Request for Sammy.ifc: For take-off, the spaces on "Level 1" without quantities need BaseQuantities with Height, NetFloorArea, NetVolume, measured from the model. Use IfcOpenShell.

First a look at what the model holds.

```python
import ifcopenshell
import ifcopenshell.util.element
import ifcopenshell.util.unit

model = ifcopenshell.open("Sammy.ifc")
print(model.schema)
for unit_type in ("LENGTHUNIT", "AREAUNIT", "VOLUMEUNIT"):
    print(unit_type, ifcopenshell.util.unit.calculate_unit_scale(model, unit_type))
storey = next(s for s in model.by_type("IfcBuildingStorey") if s.Name == "Level 1")
spaces = [e for e in ifcopenshell.util.element.get_decomposition(storey) if e.is_a("IfcSpace")]
for e in sorted(spaces, key=lambda e: e.id()):
    print(e.id(), e.is_a(), e.Name, list(ifcopenshell.util.element.get_psets(e, qtos_only=True)), sep=" | ")
```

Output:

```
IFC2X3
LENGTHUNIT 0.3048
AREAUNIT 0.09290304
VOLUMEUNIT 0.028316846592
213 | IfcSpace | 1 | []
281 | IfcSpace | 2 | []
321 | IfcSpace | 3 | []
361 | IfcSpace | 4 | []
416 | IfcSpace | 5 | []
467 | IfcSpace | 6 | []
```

```python
import ifcopenshell
import ifcopenshell.api.pset
import ifcopenshell.geom
import ifcopenshell.util.element
import ifcopenshell.util.shape
import ifcopenshell.util.unit

model = ifcopenshell.open("Sammy.ifc")
unit_scale = ifcopenshell.util.unit.calculate_unit_scale(model)
area_scale = ifcopenshell.util.unit.calculate_unit_scale(model, "AREAUNIT")
volume_scale = ifcopenshell.util.unit.calculate_unit_scale(model, "VOLUMEUNIT")
settings = ifcopenshell.geom.settings()

storey = next(s for s in model.by_type("IfcBuildingStorey") if s.Name == "Level 1")
spaces = [e for e in ifcopenshell.util.element.get_decomposition(storey) if e.is_a("IfcSpace")]

for e in sorted(spaces, key=lambda e: e.id()):
    if ifcopenshell.util.element.get_psets(e, qtos_only=True, should_inherit=False):
        continue
    # Geometry comes back in metres, in the element's own axes.
    shape = ifcopenshell.geom.create_shape(settings, e)
    values = {
        "Height": ifcopenshell.util.shape.get_z(shape.geometry) / unit_scale,
        "NetFloorArea": ifcopenshell.util.shape.get_footprint_area(shape.geometry) / area_scale,
        "NetVolume": ifcopenshell.util.shape.get_volume(shape.geometry) / volume_scale,
    }
    qto = ifcopenshell.api.pset.add_qto(model, product=e, name="BaseQuantities")
    ifcopenshell.api.pset.edit_qto(model, qto=qto, properties=values)
    print(e.id(), {k: round(v, 3) for k, v in values.items()})

model.write("Sammy_updated.ifc")
```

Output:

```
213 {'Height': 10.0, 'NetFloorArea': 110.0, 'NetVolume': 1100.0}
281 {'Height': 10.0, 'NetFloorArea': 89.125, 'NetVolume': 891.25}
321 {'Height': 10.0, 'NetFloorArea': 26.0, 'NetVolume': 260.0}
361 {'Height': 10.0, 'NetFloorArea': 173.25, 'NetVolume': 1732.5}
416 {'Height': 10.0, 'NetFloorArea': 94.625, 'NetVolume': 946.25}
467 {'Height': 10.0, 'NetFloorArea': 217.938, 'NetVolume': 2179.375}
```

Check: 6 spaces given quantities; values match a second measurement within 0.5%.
